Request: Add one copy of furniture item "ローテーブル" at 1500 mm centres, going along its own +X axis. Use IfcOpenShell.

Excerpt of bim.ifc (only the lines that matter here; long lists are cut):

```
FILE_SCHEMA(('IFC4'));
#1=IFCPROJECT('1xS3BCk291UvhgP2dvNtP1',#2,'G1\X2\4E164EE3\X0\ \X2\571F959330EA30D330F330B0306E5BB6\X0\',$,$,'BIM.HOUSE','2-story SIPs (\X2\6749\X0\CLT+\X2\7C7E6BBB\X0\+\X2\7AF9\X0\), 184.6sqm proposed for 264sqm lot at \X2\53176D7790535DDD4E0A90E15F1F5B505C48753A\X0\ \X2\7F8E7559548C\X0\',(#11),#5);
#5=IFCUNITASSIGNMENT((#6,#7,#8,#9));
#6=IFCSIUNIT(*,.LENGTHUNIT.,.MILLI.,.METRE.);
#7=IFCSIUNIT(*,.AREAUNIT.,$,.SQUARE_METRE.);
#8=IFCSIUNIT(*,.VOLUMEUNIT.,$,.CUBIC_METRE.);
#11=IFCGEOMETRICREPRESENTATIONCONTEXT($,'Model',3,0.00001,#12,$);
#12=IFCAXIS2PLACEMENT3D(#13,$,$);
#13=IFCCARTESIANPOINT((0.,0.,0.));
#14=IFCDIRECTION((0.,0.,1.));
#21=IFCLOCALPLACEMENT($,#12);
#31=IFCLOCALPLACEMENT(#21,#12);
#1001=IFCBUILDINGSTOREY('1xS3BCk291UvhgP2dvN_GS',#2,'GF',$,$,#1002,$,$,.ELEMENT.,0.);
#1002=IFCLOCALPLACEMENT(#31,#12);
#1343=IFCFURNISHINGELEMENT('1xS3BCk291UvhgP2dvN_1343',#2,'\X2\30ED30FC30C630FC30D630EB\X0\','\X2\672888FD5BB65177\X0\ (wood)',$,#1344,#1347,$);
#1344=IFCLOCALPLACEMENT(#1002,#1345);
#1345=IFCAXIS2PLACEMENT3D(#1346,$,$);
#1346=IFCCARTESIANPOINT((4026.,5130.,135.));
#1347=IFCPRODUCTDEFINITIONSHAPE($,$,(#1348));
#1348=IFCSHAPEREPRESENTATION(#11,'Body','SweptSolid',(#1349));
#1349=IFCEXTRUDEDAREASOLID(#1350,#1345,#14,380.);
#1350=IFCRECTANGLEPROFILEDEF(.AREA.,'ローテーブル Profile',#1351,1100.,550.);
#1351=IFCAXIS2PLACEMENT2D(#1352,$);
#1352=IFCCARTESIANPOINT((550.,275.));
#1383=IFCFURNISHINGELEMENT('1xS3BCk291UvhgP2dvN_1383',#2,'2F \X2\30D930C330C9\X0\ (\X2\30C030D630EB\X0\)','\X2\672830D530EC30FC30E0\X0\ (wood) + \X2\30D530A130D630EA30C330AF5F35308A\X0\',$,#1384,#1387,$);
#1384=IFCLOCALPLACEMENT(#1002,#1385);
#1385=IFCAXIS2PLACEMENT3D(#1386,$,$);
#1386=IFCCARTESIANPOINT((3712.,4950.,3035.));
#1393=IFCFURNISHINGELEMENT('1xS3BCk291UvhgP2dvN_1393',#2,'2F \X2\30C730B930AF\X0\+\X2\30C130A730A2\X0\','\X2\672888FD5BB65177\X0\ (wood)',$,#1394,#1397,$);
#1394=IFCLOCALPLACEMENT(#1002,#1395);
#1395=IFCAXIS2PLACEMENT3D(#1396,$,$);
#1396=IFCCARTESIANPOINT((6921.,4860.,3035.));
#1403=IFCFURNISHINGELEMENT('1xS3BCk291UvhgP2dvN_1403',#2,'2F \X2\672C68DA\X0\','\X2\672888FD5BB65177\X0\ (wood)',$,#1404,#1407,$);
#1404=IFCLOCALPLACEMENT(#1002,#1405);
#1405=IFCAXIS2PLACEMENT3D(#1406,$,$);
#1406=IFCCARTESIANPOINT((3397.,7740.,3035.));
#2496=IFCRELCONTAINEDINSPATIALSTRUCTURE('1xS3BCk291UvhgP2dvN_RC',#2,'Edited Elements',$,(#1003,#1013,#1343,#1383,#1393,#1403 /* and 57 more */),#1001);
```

```python
import ifcopenshell
import ifcopenshell.api.geometry
import ifcopenshell.api.root
import ifcopenshell.util.element
import ifcopenshell.util.placement
import ifcopenshell.util.unit

model = ifcopenshell.open("bim.ifc")
unit_scale = ifcopenshell.util.unit.calculate_unit_scale(model)


def reuse_history(source, copy):
    """copy_class also copies each property set's owner history, people and application; keep the originals."""
    for rel in copy.IsDefinedBy:
        if rel.is_a("IfcRelDefinesByProperties") and (history := rel.RelatingPropertyDefinition.OwnerHistory):
            rel.RelatingPropertyDefinition.OwnerHistory = source.OwnerHistory
            ifcopenshell.util.element.remove_deep2(model, history)


source = model.by_guid("1xS3BCk291UvhgP2dvN_1343")
base = ifcopenshell.util.placement.get_local_placement(source.ObjectPlacement)
step = base[:3, 0] * 1.5 / unit_scale

for i in range(1, 2):
    copy = ifcopenshell.api.root.copy_class(model, product=source)
    copy.Representation = ifcopenshell.util.element.copy_deep(
        model, source.Representation, exclude=["IfcGeometricRepresentationContext", "IfcRepresentationMap"]
    )
    reuse_history(source, copy)
    matrix = base.copy()
    matrix[:3, 3] += i * step
    print("added at", matrix[:3, 3].round(3) + 0.0)
    ifcopenshell.api.geometry.edit_object_placement(model, product=copy, matrix=matrix, is_si=False)

model.write("bim-out.ifc")
```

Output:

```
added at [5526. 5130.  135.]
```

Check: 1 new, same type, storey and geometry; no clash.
